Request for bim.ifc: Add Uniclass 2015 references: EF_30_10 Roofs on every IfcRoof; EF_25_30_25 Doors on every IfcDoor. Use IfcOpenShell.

First a look at what the model holds.

```python
import ifcopenshell

model = ifcopenshell.open("bim.ifc")
print(model.schema)
print("classifications:", [c.Name for c in model.by_type("IfcClassification")])
for ifc_class in ("IfcDoor", "IfcRoof", "IfcStair", "IfcWall", "IfcWindow"):
    print(ifc_class, len(model.by_type(ifc_class)))
```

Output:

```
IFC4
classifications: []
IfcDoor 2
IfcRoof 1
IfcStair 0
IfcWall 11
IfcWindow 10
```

```python
import ifcopenshell
import ifcopenshell.api.classification

model = ifcopenshell.open("bim.ifc")

system = ifcopenshell.api.classification.add_classification(model, classification="Uniclass 2015")

codes = {
    "IfcRoof": ("EF_30_10", "Roofs"),
    "IfcDoor": ("EF_25_30_25", "Doors"),
}
for ifc_class, (code, name) in codes.items():
    products = model.by_type(ifc_class)
    ifcopenshell.api.classification.add_reference(
        model, products=products, classification=system, identification=code, name=name
    )
    print(code, len(products))

model.write("bim_edited.ifc")
```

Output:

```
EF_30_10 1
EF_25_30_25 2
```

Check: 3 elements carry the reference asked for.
